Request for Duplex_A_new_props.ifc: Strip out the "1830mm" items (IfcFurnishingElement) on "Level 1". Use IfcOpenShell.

First a look at what the model holds.

```python
import ifcopenshell
import ifcopenshell.util.element

model = ifcopenshell.open("Duplex_A_new_props.ifc")
print(model.schema)
storey = next(s for s in model.by_type("IfcBuildingStorey") if s.Name == "Level 1")
furniture = [e for e in ifcopenshell.util.element.get_decomposition(storey) if e.is_a("IfcFurnishingElement")]
seen = {}
for e in furniture:
    element_type = ifcopenshell.util.element.get_type(e)
    name = element_type.Name if element_type not in (None, e) else None
    seen[name] = seen.get(name, 0) + 1
for name, count in sorted(seen.items(), key=str):
    print(count, "x", name)
```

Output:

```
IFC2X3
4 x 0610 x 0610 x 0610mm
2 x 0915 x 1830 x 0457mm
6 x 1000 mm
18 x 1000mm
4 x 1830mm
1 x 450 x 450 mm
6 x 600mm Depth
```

```python
import ifcopenshell
import ifcopenshell.api.root
import ifcopenshell.util.element

model = ifcopenshell.open("Duplex_A_new_props.ifc")

storey = next(s for s in model.by_type("IfcBuildingStorey") if s.Name == "Level 1")
furniture = [e for e in ifcopenshell.util.element.get_decomposition(storey) if e.is_a("IfcFurnishingElement")]
targets = [e for e in furniture if (t := ifcopenshell.util.element.get_type(e)) not in (None, e) and t.Name == "1830mm"]

for e in targets:
    ifcopenshell.api.root.remove_product(model, product=e)
print(len(targets), "removed")

model.write("Duplex_A_new_props_rev.ifc")
```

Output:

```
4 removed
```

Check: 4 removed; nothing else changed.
